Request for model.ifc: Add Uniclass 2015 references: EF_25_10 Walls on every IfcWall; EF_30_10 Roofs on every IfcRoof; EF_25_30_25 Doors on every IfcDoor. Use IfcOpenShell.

First a look at what the model holds.

```python
import ifcopenshell

model = ifcopenshell.open("model.ifc")
print(model.schema)
print("classifications:", [c.Name for c in model.by_type("IfcClassification")])
for ifc_class in ("IfcDoor", "IfcRoof", "IfcStair", "IfcWall", "IfcWindow"):
    print(ifc_class, len(model.by_type(ifc_class)))
```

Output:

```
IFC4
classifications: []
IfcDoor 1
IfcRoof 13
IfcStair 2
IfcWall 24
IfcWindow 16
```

```python
import ifcopenshell
import ifcopenshell.api.classification

model = ifcopenshell.open("model.ifc")

system = ifcopenshell.api.classification.add_classification(model, classification="Uniclass 2015")

codes = {
    "IfcWall": ("EF_25_10", "Walls"),
    "IfcRoof": ("EF_30_10", "Roofs"),
    "IfcDoor": ("EF_25_30_25", "Doors"),
}
for ifc_class, (code, name) in codes.items():
    products = model.by_type(ifc_class)
    ifcopenshell.api.classification.add_reference(
        model, products=products, classification=system, identification=code, name=name
    )
    print(code, len(products))

model.write("model_rev.ifc")
```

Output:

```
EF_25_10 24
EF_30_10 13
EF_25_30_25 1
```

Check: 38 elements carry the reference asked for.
